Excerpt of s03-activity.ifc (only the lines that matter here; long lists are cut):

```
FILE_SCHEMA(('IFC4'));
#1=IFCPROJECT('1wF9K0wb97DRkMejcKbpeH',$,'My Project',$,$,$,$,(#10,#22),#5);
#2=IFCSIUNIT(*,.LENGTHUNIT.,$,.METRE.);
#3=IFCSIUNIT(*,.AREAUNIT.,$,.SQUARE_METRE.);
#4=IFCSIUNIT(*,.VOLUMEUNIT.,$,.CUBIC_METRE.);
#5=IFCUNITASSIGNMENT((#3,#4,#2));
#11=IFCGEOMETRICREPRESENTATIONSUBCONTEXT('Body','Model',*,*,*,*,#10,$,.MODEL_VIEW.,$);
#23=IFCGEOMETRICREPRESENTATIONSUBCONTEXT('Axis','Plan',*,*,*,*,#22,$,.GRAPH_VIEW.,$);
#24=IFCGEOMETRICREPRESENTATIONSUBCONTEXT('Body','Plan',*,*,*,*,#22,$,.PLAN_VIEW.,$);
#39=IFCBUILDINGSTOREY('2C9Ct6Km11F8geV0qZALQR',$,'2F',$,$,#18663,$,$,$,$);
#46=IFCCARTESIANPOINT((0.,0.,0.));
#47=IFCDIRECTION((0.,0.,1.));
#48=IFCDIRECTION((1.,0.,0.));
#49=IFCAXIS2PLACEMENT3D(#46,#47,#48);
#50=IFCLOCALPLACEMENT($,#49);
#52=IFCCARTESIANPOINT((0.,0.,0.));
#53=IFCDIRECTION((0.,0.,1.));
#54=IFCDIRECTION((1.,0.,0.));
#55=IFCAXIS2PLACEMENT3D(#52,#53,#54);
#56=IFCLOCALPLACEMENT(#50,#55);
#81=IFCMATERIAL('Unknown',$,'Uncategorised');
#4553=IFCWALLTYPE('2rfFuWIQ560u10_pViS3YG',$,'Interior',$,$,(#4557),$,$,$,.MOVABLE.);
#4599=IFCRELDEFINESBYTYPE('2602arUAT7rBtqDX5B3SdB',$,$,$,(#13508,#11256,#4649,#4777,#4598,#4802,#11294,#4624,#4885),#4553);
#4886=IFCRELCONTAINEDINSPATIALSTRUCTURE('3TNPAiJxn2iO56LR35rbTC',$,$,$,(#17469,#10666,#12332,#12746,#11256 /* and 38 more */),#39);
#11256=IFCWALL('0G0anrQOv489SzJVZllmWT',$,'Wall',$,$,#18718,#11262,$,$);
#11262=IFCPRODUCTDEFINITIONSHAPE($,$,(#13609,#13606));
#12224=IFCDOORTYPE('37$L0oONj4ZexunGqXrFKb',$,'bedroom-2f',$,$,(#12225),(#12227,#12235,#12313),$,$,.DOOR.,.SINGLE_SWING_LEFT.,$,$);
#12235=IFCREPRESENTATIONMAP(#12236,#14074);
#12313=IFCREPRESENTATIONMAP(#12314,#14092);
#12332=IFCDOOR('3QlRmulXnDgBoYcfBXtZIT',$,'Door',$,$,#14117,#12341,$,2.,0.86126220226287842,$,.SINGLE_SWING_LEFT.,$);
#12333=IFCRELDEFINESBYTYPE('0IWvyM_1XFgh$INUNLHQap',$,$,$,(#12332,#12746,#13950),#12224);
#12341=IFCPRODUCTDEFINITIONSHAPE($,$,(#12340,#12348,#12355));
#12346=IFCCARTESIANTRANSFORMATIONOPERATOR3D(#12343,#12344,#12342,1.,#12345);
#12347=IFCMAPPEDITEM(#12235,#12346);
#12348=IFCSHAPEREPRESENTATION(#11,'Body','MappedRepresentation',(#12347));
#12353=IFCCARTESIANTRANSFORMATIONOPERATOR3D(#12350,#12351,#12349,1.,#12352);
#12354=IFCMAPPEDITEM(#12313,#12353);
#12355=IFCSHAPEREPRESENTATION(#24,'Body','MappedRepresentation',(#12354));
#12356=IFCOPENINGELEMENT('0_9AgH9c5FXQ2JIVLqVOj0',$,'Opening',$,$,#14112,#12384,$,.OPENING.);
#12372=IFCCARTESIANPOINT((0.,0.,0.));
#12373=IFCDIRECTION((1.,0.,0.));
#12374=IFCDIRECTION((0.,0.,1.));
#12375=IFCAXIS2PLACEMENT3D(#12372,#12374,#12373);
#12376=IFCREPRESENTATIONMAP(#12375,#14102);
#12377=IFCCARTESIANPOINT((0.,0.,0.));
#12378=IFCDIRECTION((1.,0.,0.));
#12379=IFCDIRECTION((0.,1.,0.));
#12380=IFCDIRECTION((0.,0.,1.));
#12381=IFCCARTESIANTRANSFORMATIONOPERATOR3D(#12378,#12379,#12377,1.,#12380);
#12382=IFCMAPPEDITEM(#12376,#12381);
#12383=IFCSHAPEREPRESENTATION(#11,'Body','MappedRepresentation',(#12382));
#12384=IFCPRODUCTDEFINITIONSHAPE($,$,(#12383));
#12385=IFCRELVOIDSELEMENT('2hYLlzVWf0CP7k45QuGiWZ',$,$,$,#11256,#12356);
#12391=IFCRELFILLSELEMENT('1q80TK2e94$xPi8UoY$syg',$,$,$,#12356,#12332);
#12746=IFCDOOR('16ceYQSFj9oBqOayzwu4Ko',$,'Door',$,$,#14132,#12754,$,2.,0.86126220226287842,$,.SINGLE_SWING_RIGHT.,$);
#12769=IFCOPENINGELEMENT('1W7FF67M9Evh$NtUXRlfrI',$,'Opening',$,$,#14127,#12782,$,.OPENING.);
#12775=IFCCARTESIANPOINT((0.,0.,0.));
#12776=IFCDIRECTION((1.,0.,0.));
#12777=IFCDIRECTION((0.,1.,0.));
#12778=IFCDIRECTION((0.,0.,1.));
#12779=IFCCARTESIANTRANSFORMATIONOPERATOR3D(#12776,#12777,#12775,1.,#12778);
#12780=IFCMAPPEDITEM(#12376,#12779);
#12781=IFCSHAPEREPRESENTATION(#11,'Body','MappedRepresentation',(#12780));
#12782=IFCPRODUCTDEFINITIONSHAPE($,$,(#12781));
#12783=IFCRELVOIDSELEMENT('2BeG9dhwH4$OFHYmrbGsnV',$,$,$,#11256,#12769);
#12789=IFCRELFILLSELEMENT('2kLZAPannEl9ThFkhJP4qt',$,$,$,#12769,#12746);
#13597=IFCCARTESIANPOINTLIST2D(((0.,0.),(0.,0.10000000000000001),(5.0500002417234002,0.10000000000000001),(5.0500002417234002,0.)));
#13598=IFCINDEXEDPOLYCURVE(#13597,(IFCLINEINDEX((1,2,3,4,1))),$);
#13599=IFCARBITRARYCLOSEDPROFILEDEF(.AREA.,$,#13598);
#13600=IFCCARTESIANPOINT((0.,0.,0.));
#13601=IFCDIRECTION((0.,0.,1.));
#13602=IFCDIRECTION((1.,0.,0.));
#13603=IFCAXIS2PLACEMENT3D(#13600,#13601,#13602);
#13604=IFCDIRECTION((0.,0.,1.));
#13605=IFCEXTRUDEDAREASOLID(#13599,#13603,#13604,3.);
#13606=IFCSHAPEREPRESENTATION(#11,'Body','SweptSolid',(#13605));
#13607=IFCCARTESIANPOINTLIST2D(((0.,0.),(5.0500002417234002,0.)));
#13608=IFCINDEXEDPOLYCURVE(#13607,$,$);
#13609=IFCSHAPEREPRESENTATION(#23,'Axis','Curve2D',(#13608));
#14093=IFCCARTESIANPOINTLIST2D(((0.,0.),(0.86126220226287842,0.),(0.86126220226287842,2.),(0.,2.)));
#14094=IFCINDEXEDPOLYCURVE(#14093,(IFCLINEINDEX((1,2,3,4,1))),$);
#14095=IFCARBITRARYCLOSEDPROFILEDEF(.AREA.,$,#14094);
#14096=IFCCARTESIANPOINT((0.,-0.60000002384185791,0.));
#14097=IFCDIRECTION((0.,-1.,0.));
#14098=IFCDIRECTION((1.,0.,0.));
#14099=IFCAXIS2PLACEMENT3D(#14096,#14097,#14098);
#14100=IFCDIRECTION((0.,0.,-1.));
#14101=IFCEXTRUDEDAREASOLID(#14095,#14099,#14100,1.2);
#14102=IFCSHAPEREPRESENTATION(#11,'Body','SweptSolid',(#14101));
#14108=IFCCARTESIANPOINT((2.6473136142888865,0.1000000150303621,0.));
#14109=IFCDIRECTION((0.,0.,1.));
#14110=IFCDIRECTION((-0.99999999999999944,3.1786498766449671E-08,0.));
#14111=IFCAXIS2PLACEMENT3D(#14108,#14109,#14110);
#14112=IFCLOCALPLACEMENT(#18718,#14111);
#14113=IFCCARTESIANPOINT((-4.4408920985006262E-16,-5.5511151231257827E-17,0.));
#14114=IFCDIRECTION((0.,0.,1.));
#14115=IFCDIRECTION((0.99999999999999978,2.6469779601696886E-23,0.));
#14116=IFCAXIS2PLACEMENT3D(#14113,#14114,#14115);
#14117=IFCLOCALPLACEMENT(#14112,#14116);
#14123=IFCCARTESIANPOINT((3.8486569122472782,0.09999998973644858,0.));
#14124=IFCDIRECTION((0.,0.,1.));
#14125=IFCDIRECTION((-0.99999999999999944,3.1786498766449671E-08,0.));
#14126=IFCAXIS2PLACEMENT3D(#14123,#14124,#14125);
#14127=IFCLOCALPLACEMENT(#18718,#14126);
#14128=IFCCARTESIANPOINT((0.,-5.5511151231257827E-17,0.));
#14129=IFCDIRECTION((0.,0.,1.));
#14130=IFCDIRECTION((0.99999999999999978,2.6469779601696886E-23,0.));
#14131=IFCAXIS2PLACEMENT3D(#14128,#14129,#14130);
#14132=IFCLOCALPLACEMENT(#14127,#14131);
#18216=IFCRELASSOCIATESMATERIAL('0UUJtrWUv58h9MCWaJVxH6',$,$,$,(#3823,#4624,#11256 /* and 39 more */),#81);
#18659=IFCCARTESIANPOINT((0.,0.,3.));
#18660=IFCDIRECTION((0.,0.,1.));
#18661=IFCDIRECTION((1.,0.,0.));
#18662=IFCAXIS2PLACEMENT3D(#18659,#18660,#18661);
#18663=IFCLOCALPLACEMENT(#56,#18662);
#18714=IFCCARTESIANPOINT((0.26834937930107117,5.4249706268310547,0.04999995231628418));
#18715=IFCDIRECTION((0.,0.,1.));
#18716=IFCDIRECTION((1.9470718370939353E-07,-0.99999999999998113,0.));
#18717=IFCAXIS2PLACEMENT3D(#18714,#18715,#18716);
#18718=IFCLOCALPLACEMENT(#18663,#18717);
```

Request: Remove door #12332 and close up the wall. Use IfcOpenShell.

```python
import ifcopenshell
import ifcopenshell.api.feature
import ifcopenshell.api.root
import ifcopenshell.geom
import ifcopenshell.util.shape

model = ifcopenshell.open("s03-activity.ifc")
settings = ifcopenshell.geom.settings()


def volume(element):
    """Net volume in cubic metres, openings subtracted."""
    shape = ifcopenshell.geom.create_shape(settings, element)
    return ifcopenshell.util.shape.get_volume(shape.geometry)


door = model.by_id(12332)
opening = door.FillsVoids[0].RelatingOpeningElement
wall = opening.VoidsElements[0].RelatingBuildingElement
before = volume(wall)

ifcopenshell.api.root.remove_product(model, product=door)
ifcopenshell.api.feature.remove_feature(model, feature=opening)

after = volume(wall)

print(f"wall volume {before:.3f} -> {after:.3f} m3")

model.write("s03-activity_edited.ifc")
```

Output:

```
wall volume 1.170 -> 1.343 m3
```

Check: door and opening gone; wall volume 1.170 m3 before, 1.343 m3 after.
